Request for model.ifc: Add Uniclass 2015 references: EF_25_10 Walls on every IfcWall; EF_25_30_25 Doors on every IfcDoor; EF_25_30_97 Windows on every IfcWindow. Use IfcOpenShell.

First a look at what the model holds.

```python
import ifcopenshell

model = ifcopenshell.open("model.ifc")
print(model.schema)
print("classifications:", [c.Name for c in model.by_type("IfcClassification")])
for ifc_class in ("IfcDoor", "IfcRoof", "IfcStair", "IfcWall", "IfcWindow"):
    print(ifc_class, len(model.by_type(ifc_class)))
```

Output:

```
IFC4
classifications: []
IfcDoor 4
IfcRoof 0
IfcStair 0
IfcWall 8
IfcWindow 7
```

```python
import ifcopenshell
import ifcopenshell.api.classification

model = ifcopenshell.open("model.ifc")

system = ifcopenshell.api.classification.add_classification(model, classification="Uniclass 2015")

codes = {
    "IfcWall": ("EF_25_10", "Walls"),
    "IfcDoor": ("EF_25_30_25", "Doors"),
    "IfcWindow": ("EF_25_30_97", "Windows"),
}
for ifc_class, (code, name) in codes.items():
    products = model.by_type(ifc_class)
    ifcopenshell.api.classification.add_reference(
        model, products=products, classification=system, identification=code, name=name
    )
    print(code, len(products))

model.write("model-out.ifc")
```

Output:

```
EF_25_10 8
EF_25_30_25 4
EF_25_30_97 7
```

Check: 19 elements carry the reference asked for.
